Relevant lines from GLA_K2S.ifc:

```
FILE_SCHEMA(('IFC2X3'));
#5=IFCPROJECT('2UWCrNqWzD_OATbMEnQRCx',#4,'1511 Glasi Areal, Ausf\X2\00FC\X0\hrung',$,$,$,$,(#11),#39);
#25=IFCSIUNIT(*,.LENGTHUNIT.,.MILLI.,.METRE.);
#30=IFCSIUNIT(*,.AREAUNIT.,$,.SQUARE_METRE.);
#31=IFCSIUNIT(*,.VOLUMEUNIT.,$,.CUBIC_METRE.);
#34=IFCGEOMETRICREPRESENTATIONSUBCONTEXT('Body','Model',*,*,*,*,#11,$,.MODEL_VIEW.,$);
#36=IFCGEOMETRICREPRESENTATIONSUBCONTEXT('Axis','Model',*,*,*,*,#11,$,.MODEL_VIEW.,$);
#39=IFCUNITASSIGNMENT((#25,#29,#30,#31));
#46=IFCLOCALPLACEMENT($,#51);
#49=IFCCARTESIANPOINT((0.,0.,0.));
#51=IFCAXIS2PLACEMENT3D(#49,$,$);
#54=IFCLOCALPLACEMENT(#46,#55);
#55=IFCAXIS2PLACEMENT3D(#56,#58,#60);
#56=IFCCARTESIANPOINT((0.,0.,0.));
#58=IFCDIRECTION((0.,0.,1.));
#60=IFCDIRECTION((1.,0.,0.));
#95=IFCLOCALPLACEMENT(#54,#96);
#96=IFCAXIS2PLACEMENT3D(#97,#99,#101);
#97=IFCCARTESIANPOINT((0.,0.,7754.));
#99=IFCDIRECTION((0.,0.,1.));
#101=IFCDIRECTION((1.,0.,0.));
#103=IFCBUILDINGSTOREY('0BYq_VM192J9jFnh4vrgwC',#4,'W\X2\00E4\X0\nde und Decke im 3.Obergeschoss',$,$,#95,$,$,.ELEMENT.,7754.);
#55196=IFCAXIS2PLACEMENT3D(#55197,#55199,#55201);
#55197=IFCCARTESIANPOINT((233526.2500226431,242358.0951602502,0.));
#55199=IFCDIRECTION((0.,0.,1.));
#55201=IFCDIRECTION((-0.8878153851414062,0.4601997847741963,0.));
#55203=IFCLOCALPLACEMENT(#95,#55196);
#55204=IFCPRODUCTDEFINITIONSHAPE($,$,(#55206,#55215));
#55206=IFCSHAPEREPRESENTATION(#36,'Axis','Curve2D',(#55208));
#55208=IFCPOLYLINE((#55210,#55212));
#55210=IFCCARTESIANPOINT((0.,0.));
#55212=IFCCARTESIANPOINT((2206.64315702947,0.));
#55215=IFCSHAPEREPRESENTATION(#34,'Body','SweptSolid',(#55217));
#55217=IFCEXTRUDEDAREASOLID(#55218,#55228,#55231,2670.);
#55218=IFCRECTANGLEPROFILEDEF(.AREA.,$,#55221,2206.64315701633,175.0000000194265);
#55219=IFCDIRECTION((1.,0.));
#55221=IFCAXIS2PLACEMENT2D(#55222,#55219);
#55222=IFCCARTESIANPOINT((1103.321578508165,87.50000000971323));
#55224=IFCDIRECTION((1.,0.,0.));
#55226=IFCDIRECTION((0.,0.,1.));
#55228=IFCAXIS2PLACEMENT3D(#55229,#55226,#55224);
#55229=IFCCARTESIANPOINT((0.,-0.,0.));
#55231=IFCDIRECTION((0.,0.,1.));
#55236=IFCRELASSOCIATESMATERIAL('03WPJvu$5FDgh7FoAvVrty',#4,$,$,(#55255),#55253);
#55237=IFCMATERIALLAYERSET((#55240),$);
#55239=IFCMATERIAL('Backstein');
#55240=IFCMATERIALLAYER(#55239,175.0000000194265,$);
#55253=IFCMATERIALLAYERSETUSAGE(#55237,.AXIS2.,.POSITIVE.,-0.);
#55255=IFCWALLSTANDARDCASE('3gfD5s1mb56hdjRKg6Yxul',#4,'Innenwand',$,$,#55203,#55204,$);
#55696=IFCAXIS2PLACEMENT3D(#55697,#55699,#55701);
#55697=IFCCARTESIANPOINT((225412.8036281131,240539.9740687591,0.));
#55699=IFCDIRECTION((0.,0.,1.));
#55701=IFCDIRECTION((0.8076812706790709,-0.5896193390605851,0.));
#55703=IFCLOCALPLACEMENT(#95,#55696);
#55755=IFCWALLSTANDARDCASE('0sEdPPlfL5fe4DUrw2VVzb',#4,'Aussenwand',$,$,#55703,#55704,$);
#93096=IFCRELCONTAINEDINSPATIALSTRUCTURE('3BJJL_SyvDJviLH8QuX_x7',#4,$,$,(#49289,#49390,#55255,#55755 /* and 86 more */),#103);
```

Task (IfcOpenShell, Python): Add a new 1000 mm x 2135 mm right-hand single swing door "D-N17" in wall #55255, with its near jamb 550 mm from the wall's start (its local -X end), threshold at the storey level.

```python
import numpy as np
import ifcopenshell
import ifcopenshell.api.feature
import ifcopenshell.api.geometry
import ifcopenshell.api.root
import ifcopenshell.api.spatial
import ifcopenshell.api.type
import ifcopenshell.geom
import ifcopenshell.util.element
import ifcopenshell.util.placement
import ifcopenshell.util.representation
import ifcopenshell.util.shape
import ifcopenshell.util.unit

model = ifcopenshell.open("GLA_K2S.ifc")
unit_scale = ifcopenshell.util.unit.calculate_unit_scale(model)
settings = ifcopenshell.geom.settings()


def volume(element):
    """Net volume in cubic metres, openings subtracted."""
    shape = ifcopenshell.geom.create_shape(settings, element)
    return ifcopenshell.util.shape.get_volume(shape.geometry)


wall = model.by_id(55255)
storey = ifcopenshell.util.element.get_container(wall, ifc_class="IfcBuildingStorey")
context = ifcopenshell.util.representation.get_context(model, "Model", "Body", "MODEL_VIEW")
before = volume(wall)

width, height, from_end, sill = 1, 2.135, 0.55, 0.0  # metres

# The wall runs along its own X axis, and the end named is its -X end.
wall_shape = ifcopenshell.geom.create_shape(settings, wall)
x, y, z = ifcopenshell.util.shape.get_vertices(wall_shape.geometry).T
start = x.min() + from_end
face, thickness = float(y.min()), float(y.max() - y.min())
wall_matrix = ifcopenshell.util.placement.get_local_placement(wall.ObjectPlacement)
level = ifcopenshell.util.placement.get_local_placement(storey.ObjectPlacement)[2, 3]


def in_wall(x, y):
    """Placement at x, y metres in the wall's axes, at sill height."""
    matrix = wall_matrix.copy()
    matrix[:, 3] = wall_matrix @ np.array([x / unit_scale, y / unit_scale, 0.0, 1.0])
    matrix[2, 3] = level + sill / unit_scale
    return matrix


# Opening: a box that overshoots both wall faces by 50 mm.
opening = ifcopenshell.api.root.create_entity(model, ifc_class="IfcOpeningElement")
box = ifcopenshell.api.geometry.add_wall_representation(
    model, context=context, length=width, height=height, thickness=thickness + 0.1
)
ifcopenshell.api.geometry.assign_representation(model, product=opening, representation=box)
ifcopenshell.api.geometry.edit_object_placement(model, product=opening, matrix=in_wall(start, face - 0.05), is_si=False)
ifcopenshell.api.feature.add_feature(model, feature=opening, element=wall)

door = ifcopenshell.api.root.create_entity(model, ifc_class="IfcDoor", name="D-N17")
door.OverallWidth, door.OverallHeight = width / unit_scale, height / unit_scale
body = ifcopenshell.api.geometry.add_door_representation(
    model,
    context=context,
    overall_width=door.OverallWidth,
    overall_height=door.OverallHeight,
    operation_type="SINGLE_SWING_RIGHT",
    lining_properties={"LiningDepth": thickness / unit_scale, "ThresholdDepth": thickness / unit_scale},
)
ifcopenshell.api.geometry.assign_representation(model, product=door, representation=body)
ifcopenshell.api.spatial.assign_container(model, products=[door], relating_structure=storey)
fills = ifcopenshell.api.feature.add_filling(model, opening=opening, element=door)
fills.OwnerHistory = door.OwnerHistory  # required in IFC2X3

# IFC2X3 keeps the operation on the door style.
style = ifcopenshell.api.root.create_entity(model, ifc_class="IfcDoorStyle", name="D-N17")
style.OperationType, style.ConstructionType = "SINGLE_SWING_RIGHT", "NOTDEFINED"
style.ParameterTakesPrecedence = style.Sizeable = False
ifcopenshell.api.type.assign_type(model, related_objects=[door], relating_type=style)

# The lining spans the wall, so the door starts at the wall face.
ifcopenshell.api.geometry.edit_object_placement(model, product=door, matrix=in_wall(start, face), is_si=False)

after = volume(wall)

print(f"wall volume {before:.3f} -> {after:.3f} m3")

model.write("GLA_K2S-out.ifc")
```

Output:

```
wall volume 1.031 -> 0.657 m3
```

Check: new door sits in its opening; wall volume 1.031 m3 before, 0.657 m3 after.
